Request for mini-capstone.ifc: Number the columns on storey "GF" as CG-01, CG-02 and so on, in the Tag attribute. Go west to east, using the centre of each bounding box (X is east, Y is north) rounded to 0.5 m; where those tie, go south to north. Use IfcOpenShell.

First a look at what the model holds.

```python
import ifcopenshell
import ifcopenshell.util.element
import ifcopenshell.util.placement

model = ifcopenshell.open("mini-capstone.ifc")
print(model.schema)
storey = next(s for s in model.by_type("IfcBuildingStorey") if s.Name == "GF")
columns = [e for e in ifcopenshell.util.element.get_decomposition(storey) if e.is_a("IfcColumn")]
for e in sorted(columns, key=lambda e: e.id()):
    origin = ifcopenshell.util.placement.get_local_placement(e.ObjectPlacement)[:3, 3]
    print(e.id(), e.Tag, e.Name, origin.round(2) + 0.0, sep=" | ")
```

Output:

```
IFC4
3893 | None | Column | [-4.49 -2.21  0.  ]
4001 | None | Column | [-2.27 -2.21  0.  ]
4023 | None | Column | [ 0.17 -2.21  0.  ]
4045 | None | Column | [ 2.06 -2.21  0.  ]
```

```python
import ifcopenshell
import ifcopenshell.geom
import ifcopenshell.util.element
import ifcopenshell.util.shape

model = ifcopenshell.open("mini-capstone.ifc")
settings = ifcopenshell.geom.settings()
settings.set("use-world-coords", True)


def centre(element):
    shape = ifcopenshell.geom.create_shape(settings, element)
    return ifcopenshell.util.shape.get_bbox_centroid(shape.geometry)


storey = next(s for s in model.by_type("IfcBuildingStorey") if s.Name == "GF")
columns = [e for e in ifcopenshell.util.element.get_decomposition(storey) if e.is_a("IfcColumn")]

# Insertion points can sit at a corner or the storey origin, so sort by the geometry (in metres).
centres = {e: centre(e) for e in columns}
columns.sort(key=lambda e: (round(centres[e][0] / 0.5), centres[e][1]))

for i, e in enumerate(columns, start=1):
    number = f"CG-{i:02d}"
    e.Tag = number
    print(e.id(), number)

model.write("mini-capstone-out.ifc")
```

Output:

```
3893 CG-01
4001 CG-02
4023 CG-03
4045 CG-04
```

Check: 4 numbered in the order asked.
